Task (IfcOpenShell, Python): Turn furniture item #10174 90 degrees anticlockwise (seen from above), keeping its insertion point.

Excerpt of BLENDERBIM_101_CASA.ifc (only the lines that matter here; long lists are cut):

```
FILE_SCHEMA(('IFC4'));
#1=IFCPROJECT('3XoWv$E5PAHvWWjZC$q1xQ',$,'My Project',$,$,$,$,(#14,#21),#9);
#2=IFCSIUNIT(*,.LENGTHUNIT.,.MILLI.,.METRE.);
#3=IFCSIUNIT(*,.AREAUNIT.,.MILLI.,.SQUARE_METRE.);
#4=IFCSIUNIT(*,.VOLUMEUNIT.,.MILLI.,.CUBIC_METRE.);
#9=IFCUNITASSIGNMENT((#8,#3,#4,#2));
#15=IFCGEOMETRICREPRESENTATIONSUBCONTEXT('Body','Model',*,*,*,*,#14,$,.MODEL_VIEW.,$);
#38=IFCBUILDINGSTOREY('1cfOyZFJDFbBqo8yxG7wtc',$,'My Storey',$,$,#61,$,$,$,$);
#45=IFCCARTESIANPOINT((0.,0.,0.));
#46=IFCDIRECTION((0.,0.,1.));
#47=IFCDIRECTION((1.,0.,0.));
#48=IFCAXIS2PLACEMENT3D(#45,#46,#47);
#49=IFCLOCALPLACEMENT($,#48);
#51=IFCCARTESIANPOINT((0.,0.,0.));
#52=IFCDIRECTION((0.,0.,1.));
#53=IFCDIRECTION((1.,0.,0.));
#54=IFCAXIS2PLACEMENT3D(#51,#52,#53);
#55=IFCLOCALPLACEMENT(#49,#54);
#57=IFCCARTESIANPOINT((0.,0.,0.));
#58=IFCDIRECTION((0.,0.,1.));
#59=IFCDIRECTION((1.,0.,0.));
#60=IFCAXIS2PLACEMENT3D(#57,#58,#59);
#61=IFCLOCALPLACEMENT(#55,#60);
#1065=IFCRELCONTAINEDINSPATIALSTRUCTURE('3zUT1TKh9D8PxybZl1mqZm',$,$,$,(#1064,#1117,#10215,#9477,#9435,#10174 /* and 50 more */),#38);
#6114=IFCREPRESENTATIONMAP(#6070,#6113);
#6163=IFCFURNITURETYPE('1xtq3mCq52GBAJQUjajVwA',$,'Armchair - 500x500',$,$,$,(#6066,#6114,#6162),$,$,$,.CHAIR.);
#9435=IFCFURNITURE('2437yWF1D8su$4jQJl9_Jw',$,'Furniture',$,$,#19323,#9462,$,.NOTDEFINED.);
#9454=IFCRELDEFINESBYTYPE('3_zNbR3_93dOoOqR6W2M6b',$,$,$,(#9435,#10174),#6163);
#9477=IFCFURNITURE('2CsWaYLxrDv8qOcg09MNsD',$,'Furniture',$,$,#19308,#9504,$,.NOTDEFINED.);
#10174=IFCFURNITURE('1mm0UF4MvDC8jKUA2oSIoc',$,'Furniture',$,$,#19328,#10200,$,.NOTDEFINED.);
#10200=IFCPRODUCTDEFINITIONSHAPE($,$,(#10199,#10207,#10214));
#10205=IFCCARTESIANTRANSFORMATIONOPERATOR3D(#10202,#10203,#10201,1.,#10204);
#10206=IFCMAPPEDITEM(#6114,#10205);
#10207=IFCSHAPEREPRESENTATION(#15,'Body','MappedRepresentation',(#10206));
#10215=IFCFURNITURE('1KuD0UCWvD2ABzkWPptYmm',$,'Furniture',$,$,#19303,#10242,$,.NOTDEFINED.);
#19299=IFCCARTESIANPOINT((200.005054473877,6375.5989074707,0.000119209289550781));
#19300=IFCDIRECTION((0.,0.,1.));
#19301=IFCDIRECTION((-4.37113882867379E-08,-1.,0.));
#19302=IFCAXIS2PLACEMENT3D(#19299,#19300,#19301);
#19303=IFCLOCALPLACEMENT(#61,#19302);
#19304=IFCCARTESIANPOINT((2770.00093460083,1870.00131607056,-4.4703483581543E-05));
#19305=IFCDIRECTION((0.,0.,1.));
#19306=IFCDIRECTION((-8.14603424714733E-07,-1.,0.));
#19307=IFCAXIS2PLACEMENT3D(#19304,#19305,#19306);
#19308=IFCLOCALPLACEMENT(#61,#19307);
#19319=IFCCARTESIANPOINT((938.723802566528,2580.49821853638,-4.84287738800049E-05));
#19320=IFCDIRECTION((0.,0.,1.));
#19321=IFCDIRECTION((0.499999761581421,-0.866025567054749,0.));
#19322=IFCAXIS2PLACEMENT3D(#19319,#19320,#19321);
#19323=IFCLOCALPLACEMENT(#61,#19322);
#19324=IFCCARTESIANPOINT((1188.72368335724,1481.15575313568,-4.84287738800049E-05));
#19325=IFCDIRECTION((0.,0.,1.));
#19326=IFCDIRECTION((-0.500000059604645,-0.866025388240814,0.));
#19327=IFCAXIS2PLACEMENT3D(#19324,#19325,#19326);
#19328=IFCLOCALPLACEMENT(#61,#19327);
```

```python
import ifcopenshell
import ifcopenshell.api.geometry
import ifcopenshell.util.placement

model = ifcopenshell.open("BLENDERBIM_101_CASA.ifc")

item = model.by_guid("1mm0UF4MvDC8jKUA2oSIoc")
matrix = ifcopenshell.util.placement.get_local_placement(item.ObjectPlacement)
matrix = matrix @ ifcopenshell.util.placement.rotation(90, "Z")
ifcopenshell.api.geometry.edit_object_placement(model, product=item, matrix=matrix, is_si=False)

print(ifcopenshell.util.placement.get_local_placement(item.ObjectPlacement).round(3) + 0.0)

model.write("BLENDERBIM_101_CASA-out.ifc")
```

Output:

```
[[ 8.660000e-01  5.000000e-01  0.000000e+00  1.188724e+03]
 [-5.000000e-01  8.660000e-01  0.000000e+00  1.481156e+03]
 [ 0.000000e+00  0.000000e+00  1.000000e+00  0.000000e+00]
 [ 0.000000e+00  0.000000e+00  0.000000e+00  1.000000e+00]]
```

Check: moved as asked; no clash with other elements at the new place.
